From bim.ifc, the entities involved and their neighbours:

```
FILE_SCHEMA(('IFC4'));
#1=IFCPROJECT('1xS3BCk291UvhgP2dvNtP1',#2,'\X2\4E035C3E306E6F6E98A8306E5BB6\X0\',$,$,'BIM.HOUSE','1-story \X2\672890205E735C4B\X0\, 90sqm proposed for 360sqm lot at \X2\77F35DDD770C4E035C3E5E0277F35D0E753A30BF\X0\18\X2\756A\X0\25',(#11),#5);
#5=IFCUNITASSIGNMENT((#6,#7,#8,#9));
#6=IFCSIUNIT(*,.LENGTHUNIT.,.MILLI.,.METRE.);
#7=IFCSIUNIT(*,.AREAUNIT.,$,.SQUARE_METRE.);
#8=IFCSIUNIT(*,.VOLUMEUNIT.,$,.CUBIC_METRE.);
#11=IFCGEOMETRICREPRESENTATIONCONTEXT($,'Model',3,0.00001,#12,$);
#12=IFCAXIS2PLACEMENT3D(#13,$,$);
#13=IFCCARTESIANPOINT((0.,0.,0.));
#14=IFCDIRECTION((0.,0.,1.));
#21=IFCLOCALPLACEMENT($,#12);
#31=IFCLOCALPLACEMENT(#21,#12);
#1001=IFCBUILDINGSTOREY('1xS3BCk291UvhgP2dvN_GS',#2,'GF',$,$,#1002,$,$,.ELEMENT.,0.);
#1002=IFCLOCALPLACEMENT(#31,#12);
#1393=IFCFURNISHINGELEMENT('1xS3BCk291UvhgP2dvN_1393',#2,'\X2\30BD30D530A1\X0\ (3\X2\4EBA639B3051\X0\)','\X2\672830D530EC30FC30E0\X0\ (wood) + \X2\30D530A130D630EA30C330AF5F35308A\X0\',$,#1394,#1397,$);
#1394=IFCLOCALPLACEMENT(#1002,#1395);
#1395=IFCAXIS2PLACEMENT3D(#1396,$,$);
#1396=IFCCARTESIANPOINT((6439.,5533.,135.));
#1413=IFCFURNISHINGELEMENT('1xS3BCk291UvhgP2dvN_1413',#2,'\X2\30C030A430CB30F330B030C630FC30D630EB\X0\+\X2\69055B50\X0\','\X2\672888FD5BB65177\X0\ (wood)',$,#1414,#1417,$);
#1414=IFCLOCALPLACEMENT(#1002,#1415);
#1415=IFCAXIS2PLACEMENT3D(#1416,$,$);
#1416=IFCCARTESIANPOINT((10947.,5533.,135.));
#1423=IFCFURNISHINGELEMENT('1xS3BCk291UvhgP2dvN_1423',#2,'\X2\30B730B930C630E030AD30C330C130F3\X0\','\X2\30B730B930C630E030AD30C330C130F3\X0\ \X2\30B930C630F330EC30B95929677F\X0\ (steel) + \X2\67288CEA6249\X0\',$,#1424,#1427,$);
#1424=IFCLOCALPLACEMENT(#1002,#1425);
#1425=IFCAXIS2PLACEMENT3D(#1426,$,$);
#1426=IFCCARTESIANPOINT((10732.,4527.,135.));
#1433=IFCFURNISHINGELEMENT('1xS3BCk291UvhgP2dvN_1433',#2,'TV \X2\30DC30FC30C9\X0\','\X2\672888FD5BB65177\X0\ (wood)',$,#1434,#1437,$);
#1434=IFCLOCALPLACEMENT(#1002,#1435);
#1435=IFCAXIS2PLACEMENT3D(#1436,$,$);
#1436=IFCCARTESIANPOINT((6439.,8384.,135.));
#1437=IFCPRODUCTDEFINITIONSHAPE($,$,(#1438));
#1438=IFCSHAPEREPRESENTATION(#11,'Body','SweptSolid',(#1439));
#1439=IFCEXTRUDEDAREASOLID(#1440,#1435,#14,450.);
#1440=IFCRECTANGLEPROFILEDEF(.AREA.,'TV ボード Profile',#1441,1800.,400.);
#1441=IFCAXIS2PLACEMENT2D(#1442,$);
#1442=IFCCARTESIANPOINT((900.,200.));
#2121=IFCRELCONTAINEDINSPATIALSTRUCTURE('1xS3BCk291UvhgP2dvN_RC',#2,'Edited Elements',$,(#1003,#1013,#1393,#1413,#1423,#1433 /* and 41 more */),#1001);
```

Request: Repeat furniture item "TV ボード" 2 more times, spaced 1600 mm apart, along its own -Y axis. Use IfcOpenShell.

```python
import ifcopenshell
import ifcopenshell.api.geometry
import ifcopenshell.api.root
import ifcopenshell.util.element
import ifcopenshell.util.placement
import ifcopenshell.util.unit

model = ifcopenshell.open("bim.ifc")
unit_scale = ifcopenshell.util.unit.calculate_unit_scale(model)


def reuse_history(source, copy):
    """copy_class also copies each property set's owner history, people and application; keep the originals."""
    for rel in copy.IsDefinedBy:
        if rel.is_a("IfcRelDefinesByProperties") and (history := rel.RelatingPropertyDefinition.OwnerHistory):
            rel.RelatingPropertyDefinition.OwnerHistory = source.OwnerHistory
            ifcopenshell.util.element.remove_deep2(model, history)


source = model.by_id(1433)
base = ifcopenshell.util.placement.get_local_placement(source.ObjectPlacement)
step = -base[:3, 1] * 1.6 / unit_scale

for i in range(1, 3):
    copy = ifcopenshell.api.root.copy_class(model, product=source)
    copy.Representation = ifcopenshell.util.element.copy_deep(
        model, source.Representation, exclude=["IfcGeometricRepresentationContext", "IfcRepresentationMap"]
    )
    reuse_history(source, copy)
    matrix = base.copy()
    matrix[:3, 3] += i * step
    print("added at", matrix[:3, 3].round(3) + 0.0)
    ifcopenshell.api.geometry.edit_object_placement(model, product=copy, matrix=matrix, is_si=False)

model.write("bim_updated.ifc")
```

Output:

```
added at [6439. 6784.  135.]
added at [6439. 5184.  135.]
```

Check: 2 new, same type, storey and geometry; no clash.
